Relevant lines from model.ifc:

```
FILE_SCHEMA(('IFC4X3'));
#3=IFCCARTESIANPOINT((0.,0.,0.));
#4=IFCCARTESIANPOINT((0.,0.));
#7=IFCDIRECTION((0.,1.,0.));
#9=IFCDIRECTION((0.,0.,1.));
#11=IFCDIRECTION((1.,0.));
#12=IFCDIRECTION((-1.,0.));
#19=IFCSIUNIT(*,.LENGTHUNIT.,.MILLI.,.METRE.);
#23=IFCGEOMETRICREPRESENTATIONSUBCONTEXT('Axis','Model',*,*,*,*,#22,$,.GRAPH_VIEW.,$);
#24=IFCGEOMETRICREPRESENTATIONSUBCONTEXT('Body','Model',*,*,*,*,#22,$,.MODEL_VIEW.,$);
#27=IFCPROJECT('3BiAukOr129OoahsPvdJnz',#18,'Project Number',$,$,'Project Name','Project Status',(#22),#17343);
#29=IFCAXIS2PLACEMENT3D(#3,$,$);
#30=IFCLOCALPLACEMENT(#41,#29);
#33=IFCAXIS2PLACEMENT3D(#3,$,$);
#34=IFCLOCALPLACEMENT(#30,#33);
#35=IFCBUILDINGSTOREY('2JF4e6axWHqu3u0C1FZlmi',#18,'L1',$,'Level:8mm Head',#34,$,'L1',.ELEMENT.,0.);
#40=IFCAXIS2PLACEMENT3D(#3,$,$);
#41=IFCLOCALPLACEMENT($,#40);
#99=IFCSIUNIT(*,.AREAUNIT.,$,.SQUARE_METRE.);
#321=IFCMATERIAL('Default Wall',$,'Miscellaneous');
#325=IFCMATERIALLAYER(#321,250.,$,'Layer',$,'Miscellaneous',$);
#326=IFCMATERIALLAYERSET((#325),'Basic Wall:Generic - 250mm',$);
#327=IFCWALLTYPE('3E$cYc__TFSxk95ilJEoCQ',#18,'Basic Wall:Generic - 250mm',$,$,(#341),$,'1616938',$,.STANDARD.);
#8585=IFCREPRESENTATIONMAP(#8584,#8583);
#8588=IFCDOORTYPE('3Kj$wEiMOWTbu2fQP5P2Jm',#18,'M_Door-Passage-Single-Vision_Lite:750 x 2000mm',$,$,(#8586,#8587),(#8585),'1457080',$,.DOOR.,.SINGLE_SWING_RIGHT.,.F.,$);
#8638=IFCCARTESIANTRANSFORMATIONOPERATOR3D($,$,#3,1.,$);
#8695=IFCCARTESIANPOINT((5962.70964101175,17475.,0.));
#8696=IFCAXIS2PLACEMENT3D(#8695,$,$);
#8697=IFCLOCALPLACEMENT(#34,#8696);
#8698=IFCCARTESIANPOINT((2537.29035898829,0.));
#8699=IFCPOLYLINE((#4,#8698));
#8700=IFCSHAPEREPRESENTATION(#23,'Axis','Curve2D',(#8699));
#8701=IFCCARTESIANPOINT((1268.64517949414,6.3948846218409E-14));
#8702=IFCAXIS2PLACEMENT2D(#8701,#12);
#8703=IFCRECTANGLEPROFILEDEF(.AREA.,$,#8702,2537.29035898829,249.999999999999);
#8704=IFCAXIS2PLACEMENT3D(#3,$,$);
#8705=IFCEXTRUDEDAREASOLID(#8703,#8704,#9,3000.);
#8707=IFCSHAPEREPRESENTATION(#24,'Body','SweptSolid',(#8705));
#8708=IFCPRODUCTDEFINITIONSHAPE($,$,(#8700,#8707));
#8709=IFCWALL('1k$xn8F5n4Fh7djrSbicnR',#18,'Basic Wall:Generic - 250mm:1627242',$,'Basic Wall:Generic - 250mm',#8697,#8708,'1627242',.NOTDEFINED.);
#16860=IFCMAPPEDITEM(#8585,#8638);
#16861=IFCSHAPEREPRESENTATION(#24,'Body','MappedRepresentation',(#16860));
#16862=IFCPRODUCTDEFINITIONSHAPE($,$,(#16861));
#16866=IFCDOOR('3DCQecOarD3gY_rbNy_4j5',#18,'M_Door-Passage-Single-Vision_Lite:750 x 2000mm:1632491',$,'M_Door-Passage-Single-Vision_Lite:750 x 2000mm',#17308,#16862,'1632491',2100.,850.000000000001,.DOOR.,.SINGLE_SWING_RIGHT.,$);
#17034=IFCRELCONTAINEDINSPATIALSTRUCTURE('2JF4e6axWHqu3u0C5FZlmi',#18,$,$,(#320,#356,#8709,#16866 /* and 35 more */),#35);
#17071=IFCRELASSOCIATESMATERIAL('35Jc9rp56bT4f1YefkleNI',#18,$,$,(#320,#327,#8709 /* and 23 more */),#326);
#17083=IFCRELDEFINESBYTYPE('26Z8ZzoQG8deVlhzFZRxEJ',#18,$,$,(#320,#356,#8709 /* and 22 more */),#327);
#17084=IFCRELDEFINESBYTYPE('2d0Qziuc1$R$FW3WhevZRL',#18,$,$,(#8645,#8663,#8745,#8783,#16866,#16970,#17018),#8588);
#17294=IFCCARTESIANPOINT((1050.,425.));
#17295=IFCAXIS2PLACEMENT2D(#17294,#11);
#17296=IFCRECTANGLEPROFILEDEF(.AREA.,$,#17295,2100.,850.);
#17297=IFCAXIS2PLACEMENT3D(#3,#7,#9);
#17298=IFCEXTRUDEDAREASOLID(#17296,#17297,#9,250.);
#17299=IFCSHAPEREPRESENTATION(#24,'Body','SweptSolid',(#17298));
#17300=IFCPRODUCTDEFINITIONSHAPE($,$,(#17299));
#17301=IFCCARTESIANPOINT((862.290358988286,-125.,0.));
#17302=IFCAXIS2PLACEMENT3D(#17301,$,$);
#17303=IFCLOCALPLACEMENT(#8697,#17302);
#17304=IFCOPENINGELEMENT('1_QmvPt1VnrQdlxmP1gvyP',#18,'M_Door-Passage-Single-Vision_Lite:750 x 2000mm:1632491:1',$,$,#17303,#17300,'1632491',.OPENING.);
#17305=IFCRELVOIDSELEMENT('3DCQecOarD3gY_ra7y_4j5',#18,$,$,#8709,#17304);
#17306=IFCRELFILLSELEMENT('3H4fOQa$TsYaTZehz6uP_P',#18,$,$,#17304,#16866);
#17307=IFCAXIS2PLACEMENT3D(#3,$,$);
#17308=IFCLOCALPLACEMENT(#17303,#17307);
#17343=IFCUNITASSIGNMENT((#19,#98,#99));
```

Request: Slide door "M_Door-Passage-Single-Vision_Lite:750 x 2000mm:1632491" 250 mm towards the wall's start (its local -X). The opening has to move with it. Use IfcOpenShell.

```python
import ifcopenshell
import ifcopenshell.api.geometry
import ifcopenshell.util.placement

model = ifcopenshell.open("model.ifc")

door = model.by_guid("3DCQecOarD3gY_rbNy_4j5")
opening = door.FillsVoids[0].RelatingOpeningElement
wall = opening.VoidsElements[0].RelatingBuildingElement

wall_matrix = ifcopenshell.util.placement.get_local_placement(wall.ObjectPlacement)
shift = wall_matrix[:3, 0] * -250.0
before = ifcopenshell.util.placement.get_local_placement(door.ObjectPlacement)[:3, 3].copy()

# The door is placed relative to its opening, so it follows when the opening moves.
matrix = ifcopenshell.util.placement.get_local_placement(opening.ObjectPlacement)
matrix[:3, 3] += shift
ifcopenshell.api.geometry.edit_object_placement(
    model, product=opening, matrix=matrix, is_si=False, should_transform_children=True
)

after = ifcopenshell.util.placement.get_local_placement(door.ObjectPlacement)[:3, 3]
print("door moved by", (after - before).round(3) + 0.0)

model.write("model_edited.ifc")
```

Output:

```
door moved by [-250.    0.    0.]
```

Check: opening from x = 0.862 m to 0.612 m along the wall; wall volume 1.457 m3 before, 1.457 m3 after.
